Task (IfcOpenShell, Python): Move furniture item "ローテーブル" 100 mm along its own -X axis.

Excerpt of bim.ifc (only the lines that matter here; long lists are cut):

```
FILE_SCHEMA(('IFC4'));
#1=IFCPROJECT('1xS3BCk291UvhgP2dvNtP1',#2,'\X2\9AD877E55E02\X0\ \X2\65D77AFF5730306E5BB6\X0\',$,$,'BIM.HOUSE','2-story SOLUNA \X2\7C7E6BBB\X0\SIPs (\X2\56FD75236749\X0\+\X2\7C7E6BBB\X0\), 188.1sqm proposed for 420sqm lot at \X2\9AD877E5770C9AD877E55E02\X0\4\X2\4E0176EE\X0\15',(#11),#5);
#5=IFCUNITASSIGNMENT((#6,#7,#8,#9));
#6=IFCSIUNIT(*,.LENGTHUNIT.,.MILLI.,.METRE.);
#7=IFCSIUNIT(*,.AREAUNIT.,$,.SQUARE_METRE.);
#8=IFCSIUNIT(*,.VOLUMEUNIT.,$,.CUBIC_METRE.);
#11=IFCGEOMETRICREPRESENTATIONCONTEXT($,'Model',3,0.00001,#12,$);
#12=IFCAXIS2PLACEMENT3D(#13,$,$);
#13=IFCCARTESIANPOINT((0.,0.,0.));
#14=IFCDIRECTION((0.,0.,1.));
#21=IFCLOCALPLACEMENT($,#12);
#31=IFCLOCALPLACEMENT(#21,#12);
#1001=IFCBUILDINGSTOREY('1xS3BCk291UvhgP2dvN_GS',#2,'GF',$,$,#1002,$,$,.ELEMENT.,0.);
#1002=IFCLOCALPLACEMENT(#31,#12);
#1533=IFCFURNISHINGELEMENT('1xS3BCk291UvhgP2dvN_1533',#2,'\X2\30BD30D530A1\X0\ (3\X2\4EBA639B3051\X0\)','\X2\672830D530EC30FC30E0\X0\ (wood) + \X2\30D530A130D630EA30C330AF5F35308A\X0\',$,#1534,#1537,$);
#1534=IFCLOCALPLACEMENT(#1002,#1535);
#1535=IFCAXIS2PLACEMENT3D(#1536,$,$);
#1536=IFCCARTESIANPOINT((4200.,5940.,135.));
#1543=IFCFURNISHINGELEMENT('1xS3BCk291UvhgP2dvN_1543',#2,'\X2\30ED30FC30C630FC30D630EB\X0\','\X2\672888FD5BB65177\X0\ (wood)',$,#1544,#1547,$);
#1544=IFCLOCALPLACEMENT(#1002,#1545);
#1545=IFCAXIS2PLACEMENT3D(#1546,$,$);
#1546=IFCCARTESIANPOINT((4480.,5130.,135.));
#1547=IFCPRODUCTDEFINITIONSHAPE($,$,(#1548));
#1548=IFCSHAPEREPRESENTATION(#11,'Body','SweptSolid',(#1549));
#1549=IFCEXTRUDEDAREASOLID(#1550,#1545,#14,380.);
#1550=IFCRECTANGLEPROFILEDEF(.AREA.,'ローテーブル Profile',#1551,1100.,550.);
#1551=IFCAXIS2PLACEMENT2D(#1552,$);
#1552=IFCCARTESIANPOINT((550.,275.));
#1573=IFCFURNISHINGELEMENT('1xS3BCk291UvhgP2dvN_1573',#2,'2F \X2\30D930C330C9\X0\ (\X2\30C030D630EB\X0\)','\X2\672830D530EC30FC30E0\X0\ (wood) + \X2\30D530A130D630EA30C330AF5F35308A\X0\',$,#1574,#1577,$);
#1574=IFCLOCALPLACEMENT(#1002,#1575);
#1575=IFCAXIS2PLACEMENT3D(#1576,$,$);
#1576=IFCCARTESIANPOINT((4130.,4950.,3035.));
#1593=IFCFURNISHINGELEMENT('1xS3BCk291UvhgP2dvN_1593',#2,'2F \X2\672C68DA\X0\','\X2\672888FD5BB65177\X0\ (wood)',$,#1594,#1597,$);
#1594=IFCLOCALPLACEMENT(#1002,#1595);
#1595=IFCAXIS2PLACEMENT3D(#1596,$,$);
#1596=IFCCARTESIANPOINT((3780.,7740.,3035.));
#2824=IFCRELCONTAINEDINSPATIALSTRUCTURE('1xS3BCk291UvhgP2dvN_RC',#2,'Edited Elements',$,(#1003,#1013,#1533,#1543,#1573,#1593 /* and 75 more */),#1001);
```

```python
import ifcopenshell
import ifcopenshell.api.geometry
import ifcopenshell.util.placement
import ifcopenshell.util.unit

model = ifcopenshell.open("bim.ifc")
unit_scale = ifcopenshell.util.unit.calculate_unit_scale(model)

item = model.by_guid("1xS3BCk291UvhgP2dvN_1543")
matrix = ifcopenshell.util.placement.get_local_placement(item.ObjectPlacement)
matrix[:3, 3] -= matrix[:3, 0] * 0.1 / unit_scale
ifcopenshell.api.geometry.edit_object_placement(model, product=item, matrix=matrix, is_si=False)

print(ifcopenshell.util.placement.get_local_placement(item.ObjectPlacement).round(3) + 0.0)

model.write("bim-out.ifc")
```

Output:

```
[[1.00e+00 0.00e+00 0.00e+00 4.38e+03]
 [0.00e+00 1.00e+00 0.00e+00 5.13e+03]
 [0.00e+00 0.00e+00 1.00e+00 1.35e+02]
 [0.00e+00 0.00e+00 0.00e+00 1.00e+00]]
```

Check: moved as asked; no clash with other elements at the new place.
